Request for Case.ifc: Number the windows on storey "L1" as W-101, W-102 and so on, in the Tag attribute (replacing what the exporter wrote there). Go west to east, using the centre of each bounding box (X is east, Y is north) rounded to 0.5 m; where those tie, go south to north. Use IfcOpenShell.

First a look at what the model holds.

```python
import ifcopenshell
import ifcopenshell.util.element
import ifcopenshell.util.placement

model = ifcopenshell.open("Case.ifc")
print(model.schema)
storey = next(s for s in model.by_type("IfcBuildingStorey") if s.Name == "L1")
windows = [e for e in ifcopenshell.util.element.get_decomposition(storey) if e.is_a("IfcWindow")]
for e in sorted(windows, key=lambda e: e.id()):
    origin = ifcopenshell.util.placement.get_local_placement(e.ObjectPlacement)[:3, 3]
    print(e.id(), e.Tag, e.Name, origin.round(2) + 0.0, sep=" | ")
```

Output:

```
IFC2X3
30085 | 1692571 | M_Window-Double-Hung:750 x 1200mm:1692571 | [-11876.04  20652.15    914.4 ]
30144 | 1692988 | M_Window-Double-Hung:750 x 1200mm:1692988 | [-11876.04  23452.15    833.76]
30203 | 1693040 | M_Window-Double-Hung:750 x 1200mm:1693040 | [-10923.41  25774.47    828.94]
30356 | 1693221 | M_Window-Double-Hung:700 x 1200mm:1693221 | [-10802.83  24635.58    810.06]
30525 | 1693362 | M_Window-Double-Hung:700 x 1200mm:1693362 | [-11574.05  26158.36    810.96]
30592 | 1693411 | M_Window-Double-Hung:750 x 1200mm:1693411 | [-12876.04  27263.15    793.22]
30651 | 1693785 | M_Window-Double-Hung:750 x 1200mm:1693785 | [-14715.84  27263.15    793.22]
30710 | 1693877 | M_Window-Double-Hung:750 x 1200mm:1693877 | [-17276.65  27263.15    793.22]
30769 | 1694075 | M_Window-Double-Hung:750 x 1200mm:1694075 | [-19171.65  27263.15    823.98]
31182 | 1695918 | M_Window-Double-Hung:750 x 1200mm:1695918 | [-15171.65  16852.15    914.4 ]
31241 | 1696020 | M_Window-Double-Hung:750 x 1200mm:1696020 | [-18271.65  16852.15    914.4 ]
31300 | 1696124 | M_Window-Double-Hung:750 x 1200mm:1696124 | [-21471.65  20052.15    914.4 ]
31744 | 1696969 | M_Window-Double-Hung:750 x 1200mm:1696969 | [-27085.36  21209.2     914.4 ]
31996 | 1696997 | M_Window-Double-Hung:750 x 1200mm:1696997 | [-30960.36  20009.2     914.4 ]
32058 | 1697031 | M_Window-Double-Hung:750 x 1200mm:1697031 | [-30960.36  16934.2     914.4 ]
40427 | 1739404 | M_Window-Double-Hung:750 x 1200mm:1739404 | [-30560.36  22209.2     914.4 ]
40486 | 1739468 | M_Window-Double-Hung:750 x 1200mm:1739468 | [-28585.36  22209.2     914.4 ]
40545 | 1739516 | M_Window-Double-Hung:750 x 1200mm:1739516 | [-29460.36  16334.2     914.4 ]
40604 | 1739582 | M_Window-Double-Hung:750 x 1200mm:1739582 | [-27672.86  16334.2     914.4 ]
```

```python
import ifcopenshell
import ifcopenshell.geom
import ifcopenshell.util.element
import ifcopenshell.util.shape

model = ifcopenshell.open("Case.ifc")
settings = ifcopenshell.geom.settings()
settings.set("use-world-coords", True)


def centre(element):
    shape = ifcopenshell.geom.create_shape(settings, element)
    return ifcopenshell.util.shape.get_bbox_centroid(shape.geometry)


storey = next(s for s in model.by_type("IfcBuildingStorey") if s.Name == "L1")
windows = [e for e in ifcopenshell.util.element.get_decomposition(storey) if e.is_a("IfcWindow")]

# Insertion points can sit at a corner or the storey origin, so sort by the geometry (in metres).
centres = {e: centre(e) for e in windows}
windows.sort(key=lambda e: (round(centres[e][0] / 0.5), centres[e][1]))

for i, e in enumerate(windows, start=1):
    number = f"W-1{i:02d}"
    e.Tag = number
    print(e.id(), number)

model.write("Case_updated.ifc")
```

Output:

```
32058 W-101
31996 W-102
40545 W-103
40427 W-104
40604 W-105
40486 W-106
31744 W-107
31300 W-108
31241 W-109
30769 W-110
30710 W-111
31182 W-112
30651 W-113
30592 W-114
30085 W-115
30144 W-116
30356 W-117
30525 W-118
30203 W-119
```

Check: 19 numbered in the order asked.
